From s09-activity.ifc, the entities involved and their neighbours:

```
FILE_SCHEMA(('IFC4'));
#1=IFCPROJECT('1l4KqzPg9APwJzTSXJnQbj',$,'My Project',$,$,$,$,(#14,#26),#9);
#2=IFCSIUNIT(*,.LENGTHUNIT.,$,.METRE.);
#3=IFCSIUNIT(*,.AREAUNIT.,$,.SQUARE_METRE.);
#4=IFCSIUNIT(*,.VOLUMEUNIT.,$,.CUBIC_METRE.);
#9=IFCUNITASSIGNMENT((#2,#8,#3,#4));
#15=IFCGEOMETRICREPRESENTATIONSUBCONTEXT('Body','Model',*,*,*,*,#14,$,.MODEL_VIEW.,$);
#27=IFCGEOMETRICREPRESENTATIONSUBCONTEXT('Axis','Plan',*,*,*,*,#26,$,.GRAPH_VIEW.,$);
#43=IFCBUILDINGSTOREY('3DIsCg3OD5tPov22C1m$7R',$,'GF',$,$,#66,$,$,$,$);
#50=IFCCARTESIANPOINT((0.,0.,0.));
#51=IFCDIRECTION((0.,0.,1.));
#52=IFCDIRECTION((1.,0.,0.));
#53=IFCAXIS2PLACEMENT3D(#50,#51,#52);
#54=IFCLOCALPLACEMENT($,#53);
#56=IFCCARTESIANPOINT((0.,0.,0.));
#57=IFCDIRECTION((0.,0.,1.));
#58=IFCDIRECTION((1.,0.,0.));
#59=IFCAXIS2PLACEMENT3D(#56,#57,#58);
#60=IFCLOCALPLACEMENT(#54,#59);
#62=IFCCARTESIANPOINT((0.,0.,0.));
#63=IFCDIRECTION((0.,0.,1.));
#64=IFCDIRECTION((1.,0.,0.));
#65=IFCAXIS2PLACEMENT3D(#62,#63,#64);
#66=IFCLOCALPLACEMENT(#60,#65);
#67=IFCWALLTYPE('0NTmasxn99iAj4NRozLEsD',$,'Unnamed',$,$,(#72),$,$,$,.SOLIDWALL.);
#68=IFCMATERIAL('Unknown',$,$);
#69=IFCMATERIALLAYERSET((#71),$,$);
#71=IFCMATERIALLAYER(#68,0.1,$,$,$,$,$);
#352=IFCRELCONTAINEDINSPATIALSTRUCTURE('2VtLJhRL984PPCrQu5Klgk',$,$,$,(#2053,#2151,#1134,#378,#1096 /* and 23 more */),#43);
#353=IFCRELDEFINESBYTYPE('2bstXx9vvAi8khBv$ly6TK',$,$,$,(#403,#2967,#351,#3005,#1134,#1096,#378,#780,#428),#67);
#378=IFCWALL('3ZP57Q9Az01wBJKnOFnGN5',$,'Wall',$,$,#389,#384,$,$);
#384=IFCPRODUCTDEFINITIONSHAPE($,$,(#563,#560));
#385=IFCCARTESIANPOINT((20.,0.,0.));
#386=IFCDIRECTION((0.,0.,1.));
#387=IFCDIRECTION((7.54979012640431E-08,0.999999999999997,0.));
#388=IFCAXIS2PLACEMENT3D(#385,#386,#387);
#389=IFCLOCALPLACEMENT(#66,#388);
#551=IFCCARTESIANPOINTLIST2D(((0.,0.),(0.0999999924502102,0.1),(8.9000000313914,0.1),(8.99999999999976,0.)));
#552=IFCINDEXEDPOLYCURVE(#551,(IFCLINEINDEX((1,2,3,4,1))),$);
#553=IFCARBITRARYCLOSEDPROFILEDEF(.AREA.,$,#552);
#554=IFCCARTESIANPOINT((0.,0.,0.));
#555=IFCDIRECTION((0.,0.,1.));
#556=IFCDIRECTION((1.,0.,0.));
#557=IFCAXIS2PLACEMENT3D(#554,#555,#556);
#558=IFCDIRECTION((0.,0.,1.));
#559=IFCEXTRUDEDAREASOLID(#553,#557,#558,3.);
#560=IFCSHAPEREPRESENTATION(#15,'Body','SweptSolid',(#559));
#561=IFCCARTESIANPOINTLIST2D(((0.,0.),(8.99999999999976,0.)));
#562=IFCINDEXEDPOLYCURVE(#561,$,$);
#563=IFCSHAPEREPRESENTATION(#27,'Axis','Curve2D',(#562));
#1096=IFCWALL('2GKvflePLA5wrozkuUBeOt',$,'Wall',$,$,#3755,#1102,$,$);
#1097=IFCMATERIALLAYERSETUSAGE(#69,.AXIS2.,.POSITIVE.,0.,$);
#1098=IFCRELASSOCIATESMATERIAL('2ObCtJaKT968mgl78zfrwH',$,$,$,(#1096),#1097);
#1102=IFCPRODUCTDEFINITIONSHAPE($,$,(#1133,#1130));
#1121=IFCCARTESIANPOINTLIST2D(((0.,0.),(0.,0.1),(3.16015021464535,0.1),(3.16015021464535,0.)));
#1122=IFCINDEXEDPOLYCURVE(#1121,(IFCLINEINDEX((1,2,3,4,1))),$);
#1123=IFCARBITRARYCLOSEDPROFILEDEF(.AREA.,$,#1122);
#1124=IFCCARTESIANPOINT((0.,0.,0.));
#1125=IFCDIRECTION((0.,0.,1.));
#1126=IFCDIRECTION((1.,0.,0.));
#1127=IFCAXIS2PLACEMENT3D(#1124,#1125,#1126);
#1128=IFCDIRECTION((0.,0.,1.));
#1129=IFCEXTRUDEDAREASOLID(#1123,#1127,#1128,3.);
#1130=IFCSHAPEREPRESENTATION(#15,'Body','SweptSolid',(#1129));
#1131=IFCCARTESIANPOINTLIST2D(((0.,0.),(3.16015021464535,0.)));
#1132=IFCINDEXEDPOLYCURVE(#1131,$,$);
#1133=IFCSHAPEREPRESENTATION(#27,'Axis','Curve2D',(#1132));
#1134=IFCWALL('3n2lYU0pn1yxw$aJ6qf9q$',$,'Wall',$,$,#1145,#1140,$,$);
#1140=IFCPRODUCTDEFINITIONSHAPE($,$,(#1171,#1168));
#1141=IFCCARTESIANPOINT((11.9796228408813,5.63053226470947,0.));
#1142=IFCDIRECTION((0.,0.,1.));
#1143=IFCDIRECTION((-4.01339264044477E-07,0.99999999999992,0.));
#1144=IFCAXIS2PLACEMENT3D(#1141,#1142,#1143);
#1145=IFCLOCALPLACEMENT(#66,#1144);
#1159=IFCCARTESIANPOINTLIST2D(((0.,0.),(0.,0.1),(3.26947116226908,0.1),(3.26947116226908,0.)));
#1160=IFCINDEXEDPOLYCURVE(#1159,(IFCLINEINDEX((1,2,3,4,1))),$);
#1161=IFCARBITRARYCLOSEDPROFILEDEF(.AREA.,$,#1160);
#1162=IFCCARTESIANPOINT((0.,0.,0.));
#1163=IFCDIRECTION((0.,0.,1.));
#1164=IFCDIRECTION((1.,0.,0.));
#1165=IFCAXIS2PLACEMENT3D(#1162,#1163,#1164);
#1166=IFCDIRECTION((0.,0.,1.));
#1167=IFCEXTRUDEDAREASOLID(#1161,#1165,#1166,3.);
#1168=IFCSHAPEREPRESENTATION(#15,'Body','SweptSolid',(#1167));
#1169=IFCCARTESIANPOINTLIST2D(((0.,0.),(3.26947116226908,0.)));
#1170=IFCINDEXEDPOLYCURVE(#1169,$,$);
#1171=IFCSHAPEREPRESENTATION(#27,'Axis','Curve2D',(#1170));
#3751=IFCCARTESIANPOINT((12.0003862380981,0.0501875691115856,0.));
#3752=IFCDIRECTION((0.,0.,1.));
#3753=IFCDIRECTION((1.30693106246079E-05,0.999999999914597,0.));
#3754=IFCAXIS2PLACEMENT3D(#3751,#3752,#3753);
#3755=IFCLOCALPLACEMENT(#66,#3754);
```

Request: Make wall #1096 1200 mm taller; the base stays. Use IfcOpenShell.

```python
import ifcopenshell
import ifcopenshell.geom
import ifcopenshell.util.representation
import ifcopenshell.util.shape

model = ifcopenshell.open("s09-activity.ifc")
settings = ifcopenshell.geom.settings()


def volume(element):
    """Net volume in cubic metres, openings subtracted."""
    shape = ifcopenshell.geom.create_shape(settings, element)
    return ifcopenshell.util.shape.get_volume(shape.geometry)


wall = model.by_id(1096)
before = volume(wall)

body = ifcopenshell.util.representation.get_representation(wall, "Model", "Body")
solid = body.Items[0]
old_height = solid.Depth
solid.Depth += 1.2
after = volume(wall)

print(f"height {old_height:g} -> {solid.Depth:g}, volume {before:.3f} -> {after:.3f} m3")

model.write("s09-activity_updated.ifc")
```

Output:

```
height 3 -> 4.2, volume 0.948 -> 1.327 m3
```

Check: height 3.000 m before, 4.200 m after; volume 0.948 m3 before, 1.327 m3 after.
